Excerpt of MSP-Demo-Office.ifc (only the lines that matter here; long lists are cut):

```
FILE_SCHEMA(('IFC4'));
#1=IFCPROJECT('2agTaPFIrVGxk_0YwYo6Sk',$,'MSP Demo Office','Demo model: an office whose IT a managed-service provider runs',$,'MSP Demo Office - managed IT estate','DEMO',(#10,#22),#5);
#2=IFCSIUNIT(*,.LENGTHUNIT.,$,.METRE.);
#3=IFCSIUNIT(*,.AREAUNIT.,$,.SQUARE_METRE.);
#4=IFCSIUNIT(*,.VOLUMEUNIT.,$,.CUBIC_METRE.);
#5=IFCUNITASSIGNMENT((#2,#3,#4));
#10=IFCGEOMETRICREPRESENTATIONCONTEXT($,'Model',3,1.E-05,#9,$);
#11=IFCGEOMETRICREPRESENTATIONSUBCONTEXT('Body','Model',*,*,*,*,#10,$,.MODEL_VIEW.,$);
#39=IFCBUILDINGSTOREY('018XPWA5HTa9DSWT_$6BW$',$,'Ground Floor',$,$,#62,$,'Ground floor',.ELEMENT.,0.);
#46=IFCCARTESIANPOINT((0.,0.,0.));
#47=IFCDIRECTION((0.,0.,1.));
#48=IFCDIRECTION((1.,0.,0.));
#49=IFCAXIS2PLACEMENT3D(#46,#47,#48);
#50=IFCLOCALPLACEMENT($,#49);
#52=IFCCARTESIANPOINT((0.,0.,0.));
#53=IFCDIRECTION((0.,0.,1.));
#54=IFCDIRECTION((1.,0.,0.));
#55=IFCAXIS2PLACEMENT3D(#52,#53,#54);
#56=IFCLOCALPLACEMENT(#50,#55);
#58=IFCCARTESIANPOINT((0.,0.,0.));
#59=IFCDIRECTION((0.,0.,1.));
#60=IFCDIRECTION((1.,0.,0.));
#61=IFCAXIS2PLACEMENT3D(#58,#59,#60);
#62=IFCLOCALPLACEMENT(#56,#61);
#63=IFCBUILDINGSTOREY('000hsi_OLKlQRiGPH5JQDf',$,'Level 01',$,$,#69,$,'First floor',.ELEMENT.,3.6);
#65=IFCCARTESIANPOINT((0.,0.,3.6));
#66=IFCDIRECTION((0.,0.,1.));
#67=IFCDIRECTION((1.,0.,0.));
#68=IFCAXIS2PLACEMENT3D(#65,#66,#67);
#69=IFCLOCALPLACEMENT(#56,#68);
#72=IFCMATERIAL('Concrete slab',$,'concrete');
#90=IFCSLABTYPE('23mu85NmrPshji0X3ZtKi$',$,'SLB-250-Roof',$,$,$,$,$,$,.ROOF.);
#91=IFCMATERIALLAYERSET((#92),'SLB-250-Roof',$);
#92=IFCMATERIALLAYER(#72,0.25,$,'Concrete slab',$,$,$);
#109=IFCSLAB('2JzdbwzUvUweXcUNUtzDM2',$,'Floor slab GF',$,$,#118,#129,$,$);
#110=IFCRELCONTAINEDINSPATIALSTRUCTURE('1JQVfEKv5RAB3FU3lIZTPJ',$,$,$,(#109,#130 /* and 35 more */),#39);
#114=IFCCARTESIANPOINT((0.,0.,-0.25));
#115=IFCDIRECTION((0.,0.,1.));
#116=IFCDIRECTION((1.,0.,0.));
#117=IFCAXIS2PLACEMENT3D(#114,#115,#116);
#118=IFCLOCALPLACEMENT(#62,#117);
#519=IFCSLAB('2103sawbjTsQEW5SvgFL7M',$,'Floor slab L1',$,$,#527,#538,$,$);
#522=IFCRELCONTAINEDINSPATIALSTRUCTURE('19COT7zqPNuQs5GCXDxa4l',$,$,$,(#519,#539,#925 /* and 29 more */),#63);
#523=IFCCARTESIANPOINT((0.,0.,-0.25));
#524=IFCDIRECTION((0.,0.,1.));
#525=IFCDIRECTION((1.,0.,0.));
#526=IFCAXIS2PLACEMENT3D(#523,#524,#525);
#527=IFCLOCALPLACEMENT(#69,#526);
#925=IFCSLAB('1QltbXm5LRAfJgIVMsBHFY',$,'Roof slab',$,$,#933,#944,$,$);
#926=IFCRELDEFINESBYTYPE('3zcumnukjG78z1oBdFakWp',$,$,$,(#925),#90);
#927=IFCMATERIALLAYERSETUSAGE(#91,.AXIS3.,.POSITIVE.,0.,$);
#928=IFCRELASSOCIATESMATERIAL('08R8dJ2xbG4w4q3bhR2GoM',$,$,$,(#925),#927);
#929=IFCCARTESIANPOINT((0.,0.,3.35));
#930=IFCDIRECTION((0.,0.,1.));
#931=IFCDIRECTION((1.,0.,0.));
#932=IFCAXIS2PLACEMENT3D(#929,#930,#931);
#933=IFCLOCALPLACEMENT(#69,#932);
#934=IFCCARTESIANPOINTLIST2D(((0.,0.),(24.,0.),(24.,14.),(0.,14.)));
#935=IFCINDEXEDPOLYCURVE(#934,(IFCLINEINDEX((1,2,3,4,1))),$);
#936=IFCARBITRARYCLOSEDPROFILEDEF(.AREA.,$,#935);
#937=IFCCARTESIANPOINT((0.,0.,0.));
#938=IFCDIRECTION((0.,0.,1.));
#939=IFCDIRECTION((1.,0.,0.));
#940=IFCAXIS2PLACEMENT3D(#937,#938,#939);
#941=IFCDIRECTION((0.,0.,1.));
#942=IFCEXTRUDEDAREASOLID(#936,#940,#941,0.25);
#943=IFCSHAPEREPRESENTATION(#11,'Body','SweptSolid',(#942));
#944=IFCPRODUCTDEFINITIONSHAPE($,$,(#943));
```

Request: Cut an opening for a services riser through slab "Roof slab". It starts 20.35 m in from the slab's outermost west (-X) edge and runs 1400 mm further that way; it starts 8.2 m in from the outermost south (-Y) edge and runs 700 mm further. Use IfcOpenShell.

```python
import numpy as np
import ifcopenshell
import ifcopenshell.api.feature
import ifcopenshell.api.geometry
import ifcopenshell.api.root
import ifcopenshell.geom
import ifcopenshell.util.placement
import ifcopenshell.util.representation
import ifcopenshell.util.shape
import ifcopenshell.util.unit

model = ifcopenshell.open("MSP-Demo-Office.ifc")
unit_scale = ifcopenshell.util.unit.calculate_unit_scale(model)
settings = ifcopenshell.geom.settings()


def volume(element):
    """Net volume in cubic metres, openings subtracted."""
    shape = ifcopenshell.geom.create_shape(settings, element)
    return ifcopenshell.util.shape.get_volume(shape.geometry)


slab = model.by_guid("1QltbXm5LRAfJgIVMsBHFY")
before = volume(slab)

# Extent in the slab's own axes, in metres. The edges named are its -X and -Y sides.
slab_shape = ifcopenshell.geom.create_shape(settings, slab)
vertices = ifcopenshell.util.shape.get_vertices(slab_shape.geometry)
x_min, y_min, bottom = vertices.min(axis=0)
top = vertices[:, 2].max()

opening = ifcopenshell.api.root.create_entity(model, ifc_class="IfcOpeningElement", name="Services riser opening", predefined_type="OPENING")
context = ifcopenshell.util.representation.get_context(model, "Model", "Body", "MODEL_VIEW")
width, depth = 1.4, 0.7
outline = [(0.0, 0.0), (width, 0.0), (width, depth), (0.0, depth), (0.0, 0.0)]
# Overshoot both faces by 50 mm so the cut is clean.
shape = ifcopenshell.api.geometry.add_slab_representation(
    model, context=context, depth=top - bottom + 0.1, polyline=outline
)
ifcopenshell.api.geometry.assign_representation(model, product=opening, representation=shape)

matrix = ifcopenshell.util.placement.get_local_placement(slab.ObjectPlacement)
matrix[:, 3] = matrix @ np.append(np.array([x_min + 20.35, y_min + 8.2, bottom - 0.05]) / unit_scale, 1.0)
ifcopenshell.api.geometry.edit_object_placement(model, product=opening, matrix=matrix, is_si=False)
ifcopenshell.api.feature.add_feature(model, feature=opening, element=slab)

after = volume(slab)

print(f"slab volume {before:.3f} -> {after:.3f} m3")

model.write("MSP-Demo-Office-out.ifc")
```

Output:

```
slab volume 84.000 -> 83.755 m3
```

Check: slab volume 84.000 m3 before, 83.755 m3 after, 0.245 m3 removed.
